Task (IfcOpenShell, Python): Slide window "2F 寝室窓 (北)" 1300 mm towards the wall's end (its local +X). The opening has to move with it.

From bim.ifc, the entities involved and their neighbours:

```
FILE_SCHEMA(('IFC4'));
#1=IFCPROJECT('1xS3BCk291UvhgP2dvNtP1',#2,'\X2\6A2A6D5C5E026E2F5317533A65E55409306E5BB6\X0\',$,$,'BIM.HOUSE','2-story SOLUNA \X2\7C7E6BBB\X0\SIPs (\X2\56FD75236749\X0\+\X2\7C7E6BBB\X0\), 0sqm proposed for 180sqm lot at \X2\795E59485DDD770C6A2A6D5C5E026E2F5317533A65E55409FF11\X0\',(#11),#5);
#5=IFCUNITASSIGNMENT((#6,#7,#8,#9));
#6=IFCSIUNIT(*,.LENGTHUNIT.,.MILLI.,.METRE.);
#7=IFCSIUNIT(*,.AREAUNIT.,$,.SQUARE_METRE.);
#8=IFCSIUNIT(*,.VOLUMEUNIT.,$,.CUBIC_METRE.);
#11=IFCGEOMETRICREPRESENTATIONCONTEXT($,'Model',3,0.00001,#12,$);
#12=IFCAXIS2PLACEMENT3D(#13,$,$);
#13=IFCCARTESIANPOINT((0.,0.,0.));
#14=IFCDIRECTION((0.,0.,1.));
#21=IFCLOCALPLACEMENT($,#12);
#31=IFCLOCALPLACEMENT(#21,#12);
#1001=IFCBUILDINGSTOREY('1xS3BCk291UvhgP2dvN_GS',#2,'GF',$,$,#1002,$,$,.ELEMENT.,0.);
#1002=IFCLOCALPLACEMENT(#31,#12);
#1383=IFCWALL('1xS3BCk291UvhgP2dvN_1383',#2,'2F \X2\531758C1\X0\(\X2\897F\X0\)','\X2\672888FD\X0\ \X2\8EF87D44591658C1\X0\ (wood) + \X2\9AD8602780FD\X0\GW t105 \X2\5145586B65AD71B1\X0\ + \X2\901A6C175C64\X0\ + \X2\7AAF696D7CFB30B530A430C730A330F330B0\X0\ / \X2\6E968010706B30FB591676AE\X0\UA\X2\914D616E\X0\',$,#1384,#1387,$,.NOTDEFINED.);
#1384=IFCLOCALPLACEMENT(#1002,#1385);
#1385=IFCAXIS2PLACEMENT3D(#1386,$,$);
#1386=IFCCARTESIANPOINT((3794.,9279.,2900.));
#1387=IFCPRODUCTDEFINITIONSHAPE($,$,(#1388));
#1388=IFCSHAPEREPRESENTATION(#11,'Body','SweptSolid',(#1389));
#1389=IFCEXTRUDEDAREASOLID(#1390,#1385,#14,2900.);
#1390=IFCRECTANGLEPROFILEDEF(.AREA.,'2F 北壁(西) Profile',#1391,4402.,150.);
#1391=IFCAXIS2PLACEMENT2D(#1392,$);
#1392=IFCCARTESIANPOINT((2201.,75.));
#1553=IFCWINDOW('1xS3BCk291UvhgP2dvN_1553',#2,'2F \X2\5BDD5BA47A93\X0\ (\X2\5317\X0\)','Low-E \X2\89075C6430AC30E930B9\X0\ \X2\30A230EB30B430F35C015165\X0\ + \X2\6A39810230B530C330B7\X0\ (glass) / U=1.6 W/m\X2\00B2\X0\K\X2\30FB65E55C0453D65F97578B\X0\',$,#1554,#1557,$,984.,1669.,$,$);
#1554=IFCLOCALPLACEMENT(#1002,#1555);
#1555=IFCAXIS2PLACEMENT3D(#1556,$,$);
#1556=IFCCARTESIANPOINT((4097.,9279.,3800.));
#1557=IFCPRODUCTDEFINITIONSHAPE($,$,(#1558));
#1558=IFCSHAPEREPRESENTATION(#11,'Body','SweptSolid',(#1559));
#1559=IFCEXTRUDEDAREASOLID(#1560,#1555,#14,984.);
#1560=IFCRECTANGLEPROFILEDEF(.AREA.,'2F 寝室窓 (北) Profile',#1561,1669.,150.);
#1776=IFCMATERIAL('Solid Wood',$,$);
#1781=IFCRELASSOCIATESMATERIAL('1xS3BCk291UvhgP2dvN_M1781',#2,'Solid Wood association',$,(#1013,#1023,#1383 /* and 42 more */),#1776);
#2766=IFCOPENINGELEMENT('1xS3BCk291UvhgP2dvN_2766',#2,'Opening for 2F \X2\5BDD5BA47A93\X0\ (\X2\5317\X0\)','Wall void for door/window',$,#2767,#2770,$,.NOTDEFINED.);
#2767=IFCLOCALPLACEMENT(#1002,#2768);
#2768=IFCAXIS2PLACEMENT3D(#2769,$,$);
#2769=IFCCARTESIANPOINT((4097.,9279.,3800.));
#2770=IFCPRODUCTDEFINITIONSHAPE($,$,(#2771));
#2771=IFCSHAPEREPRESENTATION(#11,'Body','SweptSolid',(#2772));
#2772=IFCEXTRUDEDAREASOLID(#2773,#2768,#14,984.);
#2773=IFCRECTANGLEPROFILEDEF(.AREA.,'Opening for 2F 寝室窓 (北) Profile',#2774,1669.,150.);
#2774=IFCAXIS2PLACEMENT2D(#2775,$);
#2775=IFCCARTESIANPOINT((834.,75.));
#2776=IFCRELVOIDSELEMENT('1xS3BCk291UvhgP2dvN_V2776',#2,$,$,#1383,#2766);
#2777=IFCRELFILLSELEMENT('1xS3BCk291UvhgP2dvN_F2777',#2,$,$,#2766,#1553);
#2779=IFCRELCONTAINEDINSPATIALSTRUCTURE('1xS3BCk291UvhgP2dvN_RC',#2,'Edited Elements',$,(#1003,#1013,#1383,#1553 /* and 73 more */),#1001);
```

```python
import ifcopenshell
import ifcopenshell.api.geometry
import ifcopenshell.util.placement
import ifcopenshell.util.unit

model = ifcopenshell.open("bim.ifc")
unit_scale = ifcopenshell.util.unit.calculate_unit_scale(model)

window = model.by_guid("1xS3BCk291UvhgP2dvN_1553")
opening = window.FillsVoids[0].RelatingOpeningElement
wall = opening.VoidsElements[0].RelatingBuildingElement

wall_matrix = ifcopenshell.util.placement.get_local_placement(wall.ObjectPlacement)
shift = wall_matrix[:3, 0] * 1.3 / unit_scale
before = ifcopenshell.util.placement.get_local_placement(window.ObjectPlacement)[:3, 3].copy()

# The window is not placed relative to its opening, so move both.
for product in (opening, window):
    matrix = ifcopenshell.util.placement.get_local_placement(product.ObjectPlacement)
    matrix[:3, 3] += shift
    ifcopenshell.api.geometry.edit_object_placement(model, product=product, matrix=matrix, is_si=False)

after = ifcopenshell.util.placement.get_local_placement(window.ObjectPlacement)[:3, 3]
print("window moved by", (after - before).round(3) + 0.0)

model.write("bim_rev.ifc")
```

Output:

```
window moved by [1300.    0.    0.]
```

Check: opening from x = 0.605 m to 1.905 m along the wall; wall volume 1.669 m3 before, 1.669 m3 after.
